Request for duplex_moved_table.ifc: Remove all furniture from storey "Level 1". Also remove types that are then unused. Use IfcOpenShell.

First a look at what the model holds.

```python
import ifcopenshell
import ifcopenshell.util.element

model = ifcopenshell.open("duplex_moved_table.ifc")
print(model.schema)
storey = next(s for s in model.by_type("IfcBuildingStorey") if s.Name == "Level 1")
furniture = [e for e in ifcopenshell.util.element.get_decomposition(storey) if e.is_a("IfcFurnishingElement")]
seen = {}
for e in furniture:
    element_type = ifcopenshell.util.element.get_type(e)
    name = element_type.Name if element_type not in (None, e) else None
    seen[name] = seen.get(name, 0) + 1
for name, count in sorted(seen.items(), key=str):
    print(count, "x", name)
```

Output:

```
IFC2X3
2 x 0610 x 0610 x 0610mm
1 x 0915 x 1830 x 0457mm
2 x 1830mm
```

```python
import ifcopenshell
import ifcopenshell.api.root
import ifcopenshell.util.element

model = ifcopenshell.open("duplex_moved_table.ifc")

storey = next(s for s in model.by_type("IfcBuildingStorey") if s.Name == "Level 1")
furniture = [e for e in ifcopenshell.util.element.get_decomposition(storey) if e.is_a("IfcFurnishingElement")]
types = {ifcopenshell.util.element.get_type(e) for e in furniture} - {None, *furniture}

for e in furniture:
    ifcopenshell.api.root.remove_product(model, product=e)
print(len(furniture), "removed")

unused = [t for t in types if not ifcopenshell.util.element.get_types(t)]
for t in unused:
    ifcopenshell.api.root.remove_product(model, product=t)
print(len(unused), "unused types removed")

model.write("duplex_moved_table_rev.ifc")
```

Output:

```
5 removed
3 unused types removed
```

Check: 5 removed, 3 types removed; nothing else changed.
